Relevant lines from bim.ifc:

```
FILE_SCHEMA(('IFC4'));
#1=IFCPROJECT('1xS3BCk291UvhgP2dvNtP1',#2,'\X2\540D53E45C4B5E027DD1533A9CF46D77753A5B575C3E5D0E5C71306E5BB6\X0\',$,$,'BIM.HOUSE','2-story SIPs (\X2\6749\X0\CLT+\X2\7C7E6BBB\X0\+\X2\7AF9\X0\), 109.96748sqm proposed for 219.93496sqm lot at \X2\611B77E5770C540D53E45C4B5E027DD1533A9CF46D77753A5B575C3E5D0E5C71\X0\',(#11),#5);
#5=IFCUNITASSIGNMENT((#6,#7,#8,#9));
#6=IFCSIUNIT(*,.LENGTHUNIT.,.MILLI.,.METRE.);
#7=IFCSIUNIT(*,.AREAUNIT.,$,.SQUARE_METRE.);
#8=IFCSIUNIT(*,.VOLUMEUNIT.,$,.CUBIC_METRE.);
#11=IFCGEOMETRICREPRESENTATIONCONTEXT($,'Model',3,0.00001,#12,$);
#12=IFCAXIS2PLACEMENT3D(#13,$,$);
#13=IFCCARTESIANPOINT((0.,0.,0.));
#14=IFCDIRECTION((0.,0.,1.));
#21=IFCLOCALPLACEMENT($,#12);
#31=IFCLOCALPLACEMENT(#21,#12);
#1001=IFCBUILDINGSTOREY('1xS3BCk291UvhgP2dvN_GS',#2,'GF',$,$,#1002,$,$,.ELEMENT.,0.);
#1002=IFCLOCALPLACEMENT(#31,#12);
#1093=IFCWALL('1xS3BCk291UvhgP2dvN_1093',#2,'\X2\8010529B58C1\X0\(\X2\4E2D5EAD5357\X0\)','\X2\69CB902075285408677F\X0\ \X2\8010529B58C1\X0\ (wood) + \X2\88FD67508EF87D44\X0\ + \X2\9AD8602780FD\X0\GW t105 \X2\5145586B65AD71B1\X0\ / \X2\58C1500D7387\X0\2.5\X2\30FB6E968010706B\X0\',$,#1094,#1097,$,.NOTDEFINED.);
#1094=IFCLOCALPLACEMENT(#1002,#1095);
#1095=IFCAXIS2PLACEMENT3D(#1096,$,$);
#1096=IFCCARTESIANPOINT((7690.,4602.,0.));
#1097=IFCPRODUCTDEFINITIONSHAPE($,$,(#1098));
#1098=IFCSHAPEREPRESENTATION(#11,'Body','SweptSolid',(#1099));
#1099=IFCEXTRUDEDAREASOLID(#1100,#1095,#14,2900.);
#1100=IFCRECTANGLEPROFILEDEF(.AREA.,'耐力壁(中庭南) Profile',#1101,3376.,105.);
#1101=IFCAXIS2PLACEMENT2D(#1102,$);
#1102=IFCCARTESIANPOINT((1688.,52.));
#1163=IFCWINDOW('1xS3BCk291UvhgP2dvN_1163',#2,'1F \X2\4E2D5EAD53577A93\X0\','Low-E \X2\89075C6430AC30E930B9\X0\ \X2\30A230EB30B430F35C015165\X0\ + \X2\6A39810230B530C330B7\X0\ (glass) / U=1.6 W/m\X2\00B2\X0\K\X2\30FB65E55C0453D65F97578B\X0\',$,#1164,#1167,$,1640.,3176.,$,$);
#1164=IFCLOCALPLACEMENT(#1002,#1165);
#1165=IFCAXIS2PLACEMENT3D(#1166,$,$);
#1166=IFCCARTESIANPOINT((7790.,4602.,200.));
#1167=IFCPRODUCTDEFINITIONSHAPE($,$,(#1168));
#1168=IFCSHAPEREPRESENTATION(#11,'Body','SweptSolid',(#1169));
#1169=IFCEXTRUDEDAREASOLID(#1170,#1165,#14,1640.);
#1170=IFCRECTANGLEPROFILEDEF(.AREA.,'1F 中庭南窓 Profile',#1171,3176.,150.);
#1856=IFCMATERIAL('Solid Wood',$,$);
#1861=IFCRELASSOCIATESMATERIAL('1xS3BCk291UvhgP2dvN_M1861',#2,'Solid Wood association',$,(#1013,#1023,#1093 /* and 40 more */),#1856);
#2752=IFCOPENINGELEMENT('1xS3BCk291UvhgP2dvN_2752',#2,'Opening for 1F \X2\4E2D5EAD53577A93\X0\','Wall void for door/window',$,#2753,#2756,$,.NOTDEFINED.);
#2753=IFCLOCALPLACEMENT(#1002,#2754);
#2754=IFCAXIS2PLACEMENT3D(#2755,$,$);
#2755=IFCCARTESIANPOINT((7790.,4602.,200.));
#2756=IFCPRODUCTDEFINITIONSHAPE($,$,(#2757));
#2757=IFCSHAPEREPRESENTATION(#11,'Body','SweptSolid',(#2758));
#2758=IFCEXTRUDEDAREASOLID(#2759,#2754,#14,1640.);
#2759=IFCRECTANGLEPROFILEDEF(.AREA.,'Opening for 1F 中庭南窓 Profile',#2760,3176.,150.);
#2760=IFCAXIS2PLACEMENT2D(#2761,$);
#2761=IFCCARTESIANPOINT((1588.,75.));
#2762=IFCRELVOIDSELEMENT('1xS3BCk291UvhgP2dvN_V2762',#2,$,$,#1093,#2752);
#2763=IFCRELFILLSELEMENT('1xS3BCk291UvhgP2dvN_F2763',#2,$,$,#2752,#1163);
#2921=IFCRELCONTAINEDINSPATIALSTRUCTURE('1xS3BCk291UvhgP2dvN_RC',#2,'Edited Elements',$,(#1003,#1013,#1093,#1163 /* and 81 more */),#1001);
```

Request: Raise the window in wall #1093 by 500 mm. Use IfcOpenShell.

```python
import numpy as np
import ifcopenshell
import ifcopenshell.api.geometry
import ifcopenshell.util.placement
import ifcopenshell.util.unit

model = ifcopenshell.open("bim.ifc")
unit_scale = ifcopenshell.util.unit.calculate_unit_scale(model)

window = model.by_id(1163)
opening = window.FillsVoids[0].RelatingOpeningElement
dz = 500.0

shift = np.array([0.0, 0.0, dz])
# The window is not placed relative to its opening, so move both.
for product in (opening, window):
    matrix = ifcopenshell.util.placement.get_local_placement(product.ObjectPlacement)
    matrix[:3, 3] += shift
    ifcopenshell.api.geometry.edit_object_placement(model, product=product, matrix=matrix, is_si=False)

print(f"moved by {dz * unit_scale:+.3f} m")

model.write("bim_v2.ifc")
```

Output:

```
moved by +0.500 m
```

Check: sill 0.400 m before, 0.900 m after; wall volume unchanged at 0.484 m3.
